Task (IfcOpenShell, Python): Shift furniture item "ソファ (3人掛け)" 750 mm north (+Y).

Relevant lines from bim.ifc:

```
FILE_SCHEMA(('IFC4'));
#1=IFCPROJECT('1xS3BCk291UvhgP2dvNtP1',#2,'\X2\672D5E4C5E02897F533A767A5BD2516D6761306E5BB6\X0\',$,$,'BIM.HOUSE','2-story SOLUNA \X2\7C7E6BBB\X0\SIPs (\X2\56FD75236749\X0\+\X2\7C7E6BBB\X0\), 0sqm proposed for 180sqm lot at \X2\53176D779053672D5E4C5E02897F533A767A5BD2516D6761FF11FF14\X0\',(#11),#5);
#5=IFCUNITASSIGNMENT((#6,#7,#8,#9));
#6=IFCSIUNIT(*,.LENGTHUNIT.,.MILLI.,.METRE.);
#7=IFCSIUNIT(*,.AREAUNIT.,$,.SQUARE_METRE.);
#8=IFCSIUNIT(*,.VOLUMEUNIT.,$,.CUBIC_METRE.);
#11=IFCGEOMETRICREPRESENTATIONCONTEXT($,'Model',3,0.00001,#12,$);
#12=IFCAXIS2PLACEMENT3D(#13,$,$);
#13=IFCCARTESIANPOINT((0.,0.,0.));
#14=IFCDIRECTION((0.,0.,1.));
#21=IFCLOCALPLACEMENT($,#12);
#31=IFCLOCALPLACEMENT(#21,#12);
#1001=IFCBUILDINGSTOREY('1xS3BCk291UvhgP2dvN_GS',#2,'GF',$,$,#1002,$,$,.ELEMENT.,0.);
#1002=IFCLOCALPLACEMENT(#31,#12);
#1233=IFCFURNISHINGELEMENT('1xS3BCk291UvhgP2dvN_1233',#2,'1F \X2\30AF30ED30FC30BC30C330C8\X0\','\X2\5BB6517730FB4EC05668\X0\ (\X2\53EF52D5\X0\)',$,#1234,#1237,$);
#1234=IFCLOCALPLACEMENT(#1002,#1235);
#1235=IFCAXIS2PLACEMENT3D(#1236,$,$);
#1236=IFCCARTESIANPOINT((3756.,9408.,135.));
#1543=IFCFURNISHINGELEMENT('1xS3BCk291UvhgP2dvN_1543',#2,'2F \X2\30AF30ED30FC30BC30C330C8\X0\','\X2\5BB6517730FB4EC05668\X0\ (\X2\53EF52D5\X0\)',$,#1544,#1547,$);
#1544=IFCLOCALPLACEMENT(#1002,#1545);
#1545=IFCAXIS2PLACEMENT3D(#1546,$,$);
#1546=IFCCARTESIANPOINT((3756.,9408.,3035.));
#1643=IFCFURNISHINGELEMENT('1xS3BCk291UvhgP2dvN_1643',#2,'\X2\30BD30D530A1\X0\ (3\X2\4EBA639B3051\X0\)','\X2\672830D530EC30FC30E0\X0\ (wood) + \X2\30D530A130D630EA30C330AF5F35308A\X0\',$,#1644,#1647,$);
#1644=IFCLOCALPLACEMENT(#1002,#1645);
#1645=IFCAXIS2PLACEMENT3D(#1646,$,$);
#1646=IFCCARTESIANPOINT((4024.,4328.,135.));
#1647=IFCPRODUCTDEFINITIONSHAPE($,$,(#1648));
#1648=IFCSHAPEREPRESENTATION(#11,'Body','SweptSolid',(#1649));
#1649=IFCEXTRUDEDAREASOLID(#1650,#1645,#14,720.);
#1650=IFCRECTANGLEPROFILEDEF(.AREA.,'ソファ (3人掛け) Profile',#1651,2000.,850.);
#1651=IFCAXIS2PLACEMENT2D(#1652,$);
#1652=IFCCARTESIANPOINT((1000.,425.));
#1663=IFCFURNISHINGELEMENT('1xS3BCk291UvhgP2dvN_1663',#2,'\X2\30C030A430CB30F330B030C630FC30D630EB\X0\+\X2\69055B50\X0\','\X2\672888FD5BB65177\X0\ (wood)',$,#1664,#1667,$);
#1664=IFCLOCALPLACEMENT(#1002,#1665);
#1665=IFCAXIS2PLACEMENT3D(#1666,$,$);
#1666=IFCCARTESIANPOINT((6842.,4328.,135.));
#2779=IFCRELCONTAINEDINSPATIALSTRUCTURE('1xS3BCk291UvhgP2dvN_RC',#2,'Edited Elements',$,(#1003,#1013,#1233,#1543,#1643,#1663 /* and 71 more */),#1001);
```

```python
import ifcopenshell
import ifcopenshell.api.geometry
import ifcopenshell.util.placement
import ifcopenshell.util.unit

model = ifcopenshell.open("bim.ifc")
unit_scale = ifcopenshell.util.unit.calculate_unit_scale(model)

item = model.by_guid("1xS3BCk291UvhgP2dvN_1643")
matrix = ifcopenshell.util.placement.get_local_placement(item.ObjectPlacement)
matrix[1, 3] += 0.75 / unit_scale
ifcopenshell.api.geometry.edit_object_placement(model, product=item, matrix=matrix, is_si=False)

print(ifcopenshell.util.placement.get_local_placement(item.ObjectPlacement).round(3) + 0.0)

model.write("bim_edited.ifc")
```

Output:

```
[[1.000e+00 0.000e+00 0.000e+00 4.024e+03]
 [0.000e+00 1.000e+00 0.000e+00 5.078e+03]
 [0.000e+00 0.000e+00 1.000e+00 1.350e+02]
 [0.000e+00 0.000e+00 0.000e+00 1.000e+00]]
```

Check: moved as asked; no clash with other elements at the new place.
